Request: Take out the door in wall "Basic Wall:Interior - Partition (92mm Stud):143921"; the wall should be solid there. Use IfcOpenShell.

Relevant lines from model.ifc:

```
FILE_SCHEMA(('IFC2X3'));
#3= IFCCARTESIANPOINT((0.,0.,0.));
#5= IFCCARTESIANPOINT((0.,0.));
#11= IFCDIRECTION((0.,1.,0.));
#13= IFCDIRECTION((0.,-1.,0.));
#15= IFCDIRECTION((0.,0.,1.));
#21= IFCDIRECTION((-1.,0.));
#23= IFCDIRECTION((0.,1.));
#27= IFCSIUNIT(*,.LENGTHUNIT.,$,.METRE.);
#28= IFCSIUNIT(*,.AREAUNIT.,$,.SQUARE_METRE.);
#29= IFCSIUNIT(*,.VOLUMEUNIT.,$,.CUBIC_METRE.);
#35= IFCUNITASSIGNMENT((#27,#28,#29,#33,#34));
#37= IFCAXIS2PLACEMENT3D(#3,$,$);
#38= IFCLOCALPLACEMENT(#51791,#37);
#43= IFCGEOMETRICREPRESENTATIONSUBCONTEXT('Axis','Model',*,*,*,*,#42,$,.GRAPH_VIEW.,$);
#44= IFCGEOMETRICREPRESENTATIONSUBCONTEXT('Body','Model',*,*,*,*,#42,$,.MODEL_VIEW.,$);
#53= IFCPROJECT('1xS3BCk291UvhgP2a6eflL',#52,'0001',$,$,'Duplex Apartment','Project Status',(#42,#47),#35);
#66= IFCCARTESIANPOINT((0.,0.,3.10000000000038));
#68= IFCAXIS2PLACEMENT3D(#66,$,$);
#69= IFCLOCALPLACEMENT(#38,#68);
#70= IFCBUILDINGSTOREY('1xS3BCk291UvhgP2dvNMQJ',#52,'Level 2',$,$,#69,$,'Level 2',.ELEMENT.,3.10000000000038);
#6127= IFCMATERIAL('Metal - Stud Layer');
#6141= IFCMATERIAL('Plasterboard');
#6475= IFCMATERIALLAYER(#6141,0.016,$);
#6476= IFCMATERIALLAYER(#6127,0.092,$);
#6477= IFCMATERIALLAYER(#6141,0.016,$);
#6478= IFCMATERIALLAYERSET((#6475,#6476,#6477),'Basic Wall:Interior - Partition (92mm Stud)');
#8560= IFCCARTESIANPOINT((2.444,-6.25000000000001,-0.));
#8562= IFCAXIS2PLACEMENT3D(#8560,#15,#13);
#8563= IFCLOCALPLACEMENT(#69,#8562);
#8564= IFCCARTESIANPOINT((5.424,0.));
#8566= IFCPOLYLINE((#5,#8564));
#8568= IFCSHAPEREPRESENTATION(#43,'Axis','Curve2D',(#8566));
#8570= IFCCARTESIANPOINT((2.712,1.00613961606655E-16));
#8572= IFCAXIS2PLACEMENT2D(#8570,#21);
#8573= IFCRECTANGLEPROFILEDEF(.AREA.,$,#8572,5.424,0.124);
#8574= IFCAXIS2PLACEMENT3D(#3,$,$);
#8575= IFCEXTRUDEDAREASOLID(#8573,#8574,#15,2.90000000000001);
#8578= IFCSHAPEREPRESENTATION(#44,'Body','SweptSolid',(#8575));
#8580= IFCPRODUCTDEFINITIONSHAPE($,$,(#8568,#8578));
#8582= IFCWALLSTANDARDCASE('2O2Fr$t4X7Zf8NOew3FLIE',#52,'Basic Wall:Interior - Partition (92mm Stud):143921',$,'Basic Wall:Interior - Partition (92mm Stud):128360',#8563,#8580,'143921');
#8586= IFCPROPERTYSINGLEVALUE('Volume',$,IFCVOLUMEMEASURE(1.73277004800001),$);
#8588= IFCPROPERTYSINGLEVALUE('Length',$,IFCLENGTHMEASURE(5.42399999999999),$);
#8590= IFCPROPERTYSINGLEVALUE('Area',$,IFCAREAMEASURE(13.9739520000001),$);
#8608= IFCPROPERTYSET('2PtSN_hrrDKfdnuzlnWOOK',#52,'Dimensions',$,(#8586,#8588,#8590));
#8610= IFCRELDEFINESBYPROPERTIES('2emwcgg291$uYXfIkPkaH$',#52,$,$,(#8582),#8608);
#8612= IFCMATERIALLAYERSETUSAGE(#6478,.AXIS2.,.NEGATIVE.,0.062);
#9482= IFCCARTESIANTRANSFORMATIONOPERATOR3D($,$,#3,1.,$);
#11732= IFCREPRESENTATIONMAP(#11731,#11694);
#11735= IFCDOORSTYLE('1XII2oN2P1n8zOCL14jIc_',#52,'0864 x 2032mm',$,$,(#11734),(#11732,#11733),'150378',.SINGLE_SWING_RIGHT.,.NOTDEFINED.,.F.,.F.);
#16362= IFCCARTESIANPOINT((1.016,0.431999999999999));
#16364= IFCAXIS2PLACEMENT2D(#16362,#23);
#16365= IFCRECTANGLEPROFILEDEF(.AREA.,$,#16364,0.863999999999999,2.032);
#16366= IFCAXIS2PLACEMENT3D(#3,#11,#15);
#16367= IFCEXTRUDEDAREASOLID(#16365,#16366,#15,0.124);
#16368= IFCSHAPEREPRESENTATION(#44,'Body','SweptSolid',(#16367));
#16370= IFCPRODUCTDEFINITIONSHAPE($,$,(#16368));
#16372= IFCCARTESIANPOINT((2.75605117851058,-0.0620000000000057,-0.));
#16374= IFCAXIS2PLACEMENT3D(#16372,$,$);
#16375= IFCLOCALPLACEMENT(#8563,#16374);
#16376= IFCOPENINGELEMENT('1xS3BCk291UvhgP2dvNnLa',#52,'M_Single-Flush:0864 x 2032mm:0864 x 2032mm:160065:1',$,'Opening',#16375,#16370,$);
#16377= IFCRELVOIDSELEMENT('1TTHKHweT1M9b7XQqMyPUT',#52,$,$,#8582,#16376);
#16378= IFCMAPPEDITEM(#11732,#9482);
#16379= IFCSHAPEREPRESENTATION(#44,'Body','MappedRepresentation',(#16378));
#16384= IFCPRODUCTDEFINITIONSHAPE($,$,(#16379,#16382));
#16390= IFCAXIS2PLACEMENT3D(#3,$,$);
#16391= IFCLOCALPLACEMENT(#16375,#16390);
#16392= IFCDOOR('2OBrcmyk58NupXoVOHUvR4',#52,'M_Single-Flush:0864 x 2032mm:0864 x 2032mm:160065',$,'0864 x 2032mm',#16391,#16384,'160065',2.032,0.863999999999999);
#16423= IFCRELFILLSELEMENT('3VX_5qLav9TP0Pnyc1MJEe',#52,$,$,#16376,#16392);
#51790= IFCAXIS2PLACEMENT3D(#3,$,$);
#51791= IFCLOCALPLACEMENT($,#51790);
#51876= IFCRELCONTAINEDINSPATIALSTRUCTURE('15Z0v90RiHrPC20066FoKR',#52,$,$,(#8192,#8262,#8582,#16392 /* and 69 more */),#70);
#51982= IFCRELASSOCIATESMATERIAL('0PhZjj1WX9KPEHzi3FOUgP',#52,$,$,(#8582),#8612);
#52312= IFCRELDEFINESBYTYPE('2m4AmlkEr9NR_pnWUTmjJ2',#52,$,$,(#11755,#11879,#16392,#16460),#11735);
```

```python
import ifcopenshell
import ifcopenshell.api.feature
import ifcopenshell.api.pset
import ifcopenshell.api.root
import ifcopenshell.geom
import ifcopenshell.util.element
import ifcopenshell.util.shape
import ifcopenshell.util.unit

model = ifcopenshell.open("model.ifc")
area_scale = ifcopenshell.util.unit.calculate_unit_scale(model, "AREAUNIT")
volume_scale = ifcopenshell.util.unit.calculate_unit_scale(model, "VOLUMEUNIT")
settings = ifcopenshell.geom.settings()


def volume(element):
    """Net volume in cubic metres, openings subtracted."""
    shape = ifcopenshell.geom.create_shape(settings, element)
    return ifcopenshell.util.shape.get_volume(shape.geometry)


door = model.by_guid("2OBrcmyk58NupXoVOHUvR4")
opening = door.FillsVoids[0].RelatingOpeningElement
wall = opening.VoidsElements[0].RelatingBuildingElement
before = volume(wall)

ifcopenshell.api.root.remove_product(model, product=door)
ifcopenshell.api.feature.remove_feature(model, feature=opening)

after = volume(wall)
thickness = 0.124  # wall thickness in metres

# Update the wall's stored quantities.
pset = model.by_id(ifcopenshell.util.element.get_pset(wall, "Dimensions", should_inherit=False)["id"])
ifcopenshell.api.pset.edit_pset(model, pset=pset, properties={
    "Volume": model.create_entity("IfcVolumeMeasure", after / volume_scale),
    "Area": model.create_entity("IfcAreaMeasure", after / thickness / area_scale),
})

print(f"wall volume {before:.3f} -> {after:.3f} m3")

model.write("model-out.ifc")
```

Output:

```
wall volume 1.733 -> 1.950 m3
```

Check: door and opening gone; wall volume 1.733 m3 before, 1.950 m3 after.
